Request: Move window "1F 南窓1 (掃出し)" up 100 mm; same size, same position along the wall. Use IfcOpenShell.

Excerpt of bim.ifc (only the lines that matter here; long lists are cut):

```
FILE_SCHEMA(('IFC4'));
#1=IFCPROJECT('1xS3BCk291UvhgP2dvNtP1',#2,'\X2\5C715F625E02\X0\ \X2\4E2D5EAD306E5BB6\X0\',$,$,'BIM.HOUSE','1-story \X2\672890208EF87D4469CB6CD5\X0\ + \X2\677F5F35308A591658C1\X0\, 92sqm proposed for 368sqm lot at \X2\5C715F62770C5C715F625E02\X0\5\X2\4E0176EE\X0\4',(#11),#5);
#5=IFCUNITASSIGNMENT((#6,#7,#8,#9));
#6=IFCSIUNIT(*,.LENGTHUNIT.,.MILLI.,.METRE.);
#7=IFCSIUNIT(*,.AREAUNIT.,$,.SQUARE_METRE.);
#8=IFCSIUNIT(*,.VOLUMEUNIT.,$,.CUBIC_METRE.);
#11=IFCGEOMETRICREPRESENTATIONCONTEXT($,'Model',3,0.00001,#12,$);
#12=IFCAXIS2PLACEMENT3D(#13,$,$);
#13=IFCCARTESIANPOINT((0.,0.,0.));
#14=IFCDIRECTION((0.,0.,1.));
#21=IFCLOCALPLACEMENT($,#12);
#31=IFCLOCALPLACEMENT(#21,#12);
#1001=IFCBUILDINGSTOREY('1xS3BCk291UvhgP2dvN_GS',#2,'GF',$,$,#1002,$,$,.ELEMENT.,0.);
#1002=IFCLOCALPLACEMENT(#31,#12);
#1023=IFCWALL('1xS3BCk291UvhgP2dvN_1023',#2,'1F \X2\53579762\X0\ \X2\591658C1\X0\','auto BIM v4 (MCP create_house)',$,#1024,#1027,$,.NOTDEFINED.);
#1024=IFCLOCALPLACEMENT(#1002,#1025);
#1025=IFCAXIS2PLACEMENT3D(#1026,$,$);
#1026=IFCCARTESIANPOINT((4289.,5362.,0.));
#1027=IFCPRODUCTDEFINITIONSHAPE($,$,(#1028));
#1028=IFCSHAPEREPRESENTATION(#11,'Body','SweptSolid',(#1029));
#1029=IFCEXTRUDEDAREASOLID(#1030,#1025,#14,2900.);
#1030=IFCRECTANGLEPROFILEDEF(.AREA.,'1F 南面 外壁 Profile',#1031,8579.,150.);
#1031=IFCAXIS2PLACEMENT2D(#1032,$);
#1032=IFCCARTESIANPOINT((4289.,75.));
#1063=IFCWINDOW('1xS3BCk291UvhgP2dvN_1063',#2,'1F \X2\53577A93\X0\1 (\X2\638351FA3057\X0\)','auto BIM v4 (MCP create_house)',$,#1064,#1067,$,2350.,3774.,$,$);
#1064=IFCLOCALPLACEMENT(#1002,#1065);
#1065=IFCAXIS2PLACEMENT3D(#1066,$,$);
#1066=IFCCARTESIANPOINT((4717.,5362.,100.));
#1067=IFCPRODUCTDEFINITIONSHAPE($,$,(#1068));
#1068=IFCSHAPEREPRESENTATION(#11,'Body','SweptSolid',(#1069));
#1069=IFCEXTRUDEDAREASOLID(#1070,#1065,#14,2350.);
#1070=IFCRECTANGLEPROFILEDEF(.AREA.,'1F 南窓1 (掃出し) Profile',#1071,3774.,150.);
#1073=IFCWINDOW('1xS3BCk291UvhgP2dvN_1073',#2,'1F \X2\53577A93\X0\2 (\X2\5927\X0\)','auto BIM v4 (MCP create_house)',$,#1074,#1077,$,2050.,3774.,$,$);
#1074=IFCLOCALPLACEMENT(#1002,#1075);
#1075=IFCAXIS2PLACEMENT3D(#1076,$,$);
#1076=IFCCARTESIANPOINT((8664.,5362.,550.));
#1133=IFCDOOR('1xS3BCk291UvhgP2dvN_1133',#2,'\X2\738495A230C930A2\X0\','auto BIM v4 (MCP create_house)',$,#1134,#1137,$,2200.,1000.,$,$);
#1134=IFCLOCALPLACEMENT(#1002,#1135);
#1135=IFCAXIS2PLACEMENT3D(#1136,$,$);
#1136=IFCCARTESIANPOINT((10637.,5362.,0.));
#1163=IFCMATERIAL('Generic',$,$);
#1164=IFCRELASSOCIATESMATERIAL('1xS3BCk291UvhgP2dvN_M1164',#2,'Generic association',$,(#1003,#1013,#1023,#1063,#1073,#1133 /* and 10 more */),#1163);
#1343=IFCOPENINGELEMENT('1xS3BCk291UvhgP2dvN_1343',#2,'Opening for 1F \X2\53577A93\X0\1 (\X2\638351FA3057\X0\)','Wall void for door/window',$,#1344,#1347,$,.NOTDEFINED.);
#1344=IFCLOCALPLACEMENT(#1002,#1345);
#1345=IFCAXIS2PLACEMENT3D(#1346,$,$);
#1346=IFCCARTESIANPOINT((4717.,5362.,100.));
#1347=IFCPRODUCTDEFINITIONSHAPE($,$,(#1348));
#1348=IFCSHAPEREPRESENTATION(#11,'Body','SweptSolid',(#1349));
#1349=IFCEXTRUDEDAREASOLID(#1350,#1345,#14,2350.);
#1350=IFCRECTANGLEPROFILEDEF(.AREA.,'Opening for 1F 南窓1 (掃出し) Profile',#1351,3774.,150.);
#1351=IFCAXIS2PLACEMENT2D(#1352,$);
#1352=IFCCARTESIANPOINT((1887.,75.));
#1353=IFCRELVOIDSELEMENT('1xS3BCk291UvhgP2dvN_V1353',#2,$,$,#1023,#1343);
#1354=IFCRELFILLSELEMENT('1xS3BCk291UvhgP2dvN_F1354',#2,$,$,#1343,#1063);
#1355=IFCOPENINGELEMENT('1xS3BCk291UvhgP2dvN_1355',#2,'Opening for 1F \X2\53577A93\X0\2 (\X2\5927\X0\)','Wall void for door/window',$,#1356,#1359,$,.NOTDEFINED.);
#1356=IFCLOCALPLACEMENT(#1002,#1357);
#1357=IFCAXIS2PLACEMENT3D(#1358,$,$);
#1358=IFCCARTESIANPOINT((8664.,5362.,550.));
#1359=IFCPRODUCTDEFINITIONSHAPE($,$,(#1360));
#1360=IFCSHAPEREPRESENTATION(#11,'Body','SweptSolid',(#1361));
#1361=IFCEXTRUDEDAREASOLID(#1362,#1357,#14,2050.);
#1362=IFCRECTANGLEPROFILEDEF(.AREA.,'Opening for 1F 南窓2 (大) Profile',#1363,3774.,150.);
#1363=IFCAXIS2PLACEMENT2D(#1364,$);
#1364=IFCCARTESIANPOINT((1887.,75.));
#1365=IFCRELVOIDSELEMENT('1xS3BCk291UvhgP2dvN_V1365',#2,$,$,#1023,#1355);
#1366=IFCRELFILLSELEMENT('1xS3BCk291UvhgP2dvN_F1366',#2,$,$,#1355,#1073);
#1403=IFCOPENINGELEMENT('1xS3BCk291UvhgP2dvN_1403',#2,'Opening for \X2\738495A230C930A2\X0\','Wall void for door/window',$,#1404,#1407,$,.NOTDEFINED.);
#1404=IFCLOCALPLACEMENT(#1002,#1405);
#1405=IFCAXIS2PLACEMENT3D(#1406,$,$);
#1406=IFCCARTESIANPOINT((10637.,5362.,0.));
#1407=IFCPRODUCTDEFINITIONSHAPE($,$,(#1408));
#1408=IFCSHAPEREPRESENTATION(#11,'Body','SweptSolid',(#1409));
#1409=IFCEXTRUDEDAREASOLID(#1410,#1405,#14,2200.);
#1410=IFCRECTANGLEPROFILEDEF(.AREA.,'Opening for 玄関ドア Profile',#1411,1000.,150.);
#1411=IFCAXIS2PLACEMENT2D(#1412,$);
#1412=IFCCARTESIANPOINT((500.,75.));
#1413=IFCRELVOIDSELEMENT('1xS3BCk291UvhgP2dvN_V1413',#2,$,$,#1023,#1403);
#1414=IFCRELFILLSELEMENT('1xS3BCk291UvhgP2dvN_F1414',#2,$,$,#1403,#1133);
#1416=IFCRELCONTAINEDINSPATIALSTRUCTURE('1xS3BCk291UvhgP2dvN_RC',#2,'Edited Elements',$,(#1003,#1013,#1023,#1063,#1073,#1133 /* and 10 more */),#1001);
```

```python
import numpy as np
import ifcopenshell
import ifcopenshell.api.geometry
import ifcopenshell.util.placement
import ifcopenshell.util.unit

model = ifcopenshell.open("bim.ifc")
unit_scale = ifcopenshell.util.unit.calculate_unit_scale(model)

window = model.by_guid("1xS3BCk291UvhgP2dvN_1063")
opening = window.FillsVoids[0].RelatingOpeningElement
dz = 0.1 / unit_scale

shift = np.array([0.0, 0.0, dz])
# The window is not placed relative to its opening, so move both.
for product in (opening, window):
    matrix = ifcopenshell.util.placement.get_local_placement(product.ObjectPlacement)
    matrix[:3, 3] += shift
    ifcopenshell.api.geometry.edit_object_placement(model, product=product, matrix=matrix, is_si=False)

print(f"moved by {dz * unit_scale:+.3f} m")

model.write("bim-out.ifc")
```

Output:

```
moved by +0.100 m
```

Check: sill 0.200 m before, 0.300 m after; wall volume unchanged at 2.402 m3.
